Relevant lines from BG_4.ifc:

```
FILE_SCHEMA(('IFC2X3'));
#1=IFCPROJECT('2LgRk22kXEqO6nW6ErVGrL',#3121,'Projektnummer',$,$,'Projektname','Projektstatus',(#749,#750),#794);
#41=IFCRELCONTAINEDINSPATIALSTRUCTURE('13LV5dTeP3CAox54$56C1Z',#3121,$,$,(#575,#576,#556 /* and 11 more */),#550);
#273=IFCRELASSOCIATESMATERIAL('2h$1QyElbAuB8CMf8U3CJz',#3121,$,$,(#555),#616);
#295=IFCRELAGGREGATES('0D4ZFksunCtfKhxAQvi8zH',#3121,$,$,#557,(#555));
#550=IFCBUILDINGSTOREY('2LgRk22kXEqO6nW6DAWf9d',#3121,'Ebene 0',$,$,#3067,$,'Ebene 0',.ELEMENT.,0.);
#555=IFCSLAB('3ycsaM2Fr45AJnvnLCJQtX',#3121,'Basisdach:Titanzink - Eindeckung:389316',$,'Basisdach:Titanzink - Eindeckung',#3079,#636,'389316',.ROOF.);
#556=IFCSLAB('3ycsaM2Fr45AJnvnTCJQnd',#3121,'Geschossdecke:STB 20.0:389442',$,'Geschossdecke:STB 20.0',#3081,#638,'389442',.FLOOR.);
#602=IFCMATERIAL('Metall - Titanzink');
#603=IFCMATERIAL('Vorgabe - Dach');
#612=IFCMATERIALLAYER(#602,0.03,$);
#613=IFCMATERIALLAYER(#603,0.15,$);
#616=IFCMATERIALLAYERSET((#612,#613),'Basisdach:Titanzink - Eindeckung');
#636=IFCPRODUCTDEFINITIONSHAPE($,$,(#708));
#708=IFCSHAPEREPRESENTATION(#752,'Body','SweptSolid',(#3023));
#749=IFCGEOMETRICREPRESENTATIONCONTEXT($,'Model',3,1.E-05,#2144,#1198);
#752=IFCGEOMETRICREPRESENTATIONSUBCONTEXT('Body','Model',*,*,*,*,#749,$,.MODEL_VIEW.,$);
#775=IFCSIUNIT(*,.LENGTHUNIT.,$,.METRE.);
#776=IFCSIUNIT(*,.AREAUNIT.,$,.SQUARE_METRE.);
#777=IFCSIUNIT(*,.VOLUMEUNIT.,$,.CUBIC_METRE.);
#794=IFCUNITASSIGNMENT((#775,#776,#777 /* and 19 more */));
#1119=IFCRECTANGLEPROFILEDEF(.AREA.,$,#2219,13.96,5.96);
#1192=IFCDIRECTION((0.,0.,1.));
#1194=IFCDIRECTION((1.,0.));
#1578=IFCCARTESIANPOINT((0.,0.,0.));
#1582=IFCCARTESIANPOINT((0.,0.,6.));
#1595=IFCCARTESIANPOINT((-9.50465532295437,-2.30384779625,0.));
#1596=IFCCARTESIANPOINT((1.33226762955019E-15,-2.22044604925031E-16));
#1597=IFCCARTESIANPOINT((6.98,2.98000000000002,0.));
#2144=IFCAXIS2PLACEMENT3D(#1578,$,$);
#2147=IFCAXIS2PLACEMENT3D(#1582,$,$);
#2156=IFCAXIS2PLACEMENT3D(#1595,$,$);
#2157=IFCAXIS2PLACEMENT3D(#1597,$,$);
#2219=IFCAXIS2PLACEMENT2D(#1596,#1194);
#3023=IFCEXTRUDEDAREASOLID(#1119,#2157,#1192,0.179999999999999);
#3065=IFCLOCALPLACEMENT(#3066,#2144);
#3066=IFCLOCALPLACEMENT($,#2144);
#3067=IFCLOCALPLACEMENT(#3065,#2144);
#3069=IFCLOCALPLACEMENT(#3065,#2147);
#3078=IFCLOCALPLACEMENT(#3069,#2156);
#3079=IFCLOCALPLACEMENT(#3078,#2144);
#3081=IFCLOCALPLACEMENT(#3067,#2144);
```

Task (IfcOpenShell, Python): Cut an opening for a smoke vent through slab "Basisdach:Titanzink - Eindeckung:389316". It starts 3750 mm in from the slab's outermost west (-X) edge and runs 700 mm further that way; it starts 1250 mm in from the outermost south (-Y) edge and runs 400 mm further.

```python
import numpy as np
import ifcopenshell
import ifcopenshell.api.feature
import ifcopenshell.api.geometry
import ifcopenshell.api.root
import ifcopenshell.geom
import ifcopenshell.util.placement
import ifcopenshell.util.representation
import ifcopenshell.util.shape
import ifcopenshell.util.unit

model = ifcopenshell.open("BG_4.ifc")
unit_scale = ifcopenshell.util.unit.calculate_unit_scale(model)
settings = ifcopenshell.geom.settings()


def volume(element):
    """Net volume in cubic metres, openings subtracted."""
    shape = ifcopenshell.geom.create_shape(settings, element)
    return ifcopenshell.util.shape.get_volume(shape.geometry)


slab = model.by_guid("3ycsaM2Fr45AJnvnLCJQtX")
before = volume(slab)

# Extent in the slab's own axes, in metres. The edges named are its -X and -Y sides.
slab_shape = ifcopenshell.geom.create_shape(settings, slab)
vertices = ifcopenshell.util.shape.get_vertices(slab_shape.geometry)
x_min, y_min, bottom = vertices.min(axis=0)
top = vertices[:, 2].max()

opening = ifcopenshell.api.root.create_entity(model, ifc_class="IfcOpeningElement", name="Smoke vent opening")
context = ifcopenshell.util.representation.get_context(model, "Model", "Body", "MODEL_VIEW")
width, depth = 0.7, 0.4
outline = [(0.0, 0.0), (width, 0.0), (width, depth), (0.0, depth), (0.0, 0.0)]
# Overshoot both faces by 50 mm so the cut is clean.
shape = ifcopenshell.api.geometry.add_slab_representation(
    model, context=context, depth=top - bottom + 0.1, polyline=outline
)
ifcopenshell.api.geometry.assign_representation(model, product=opening, representation=shape)

matrix = ifcopenshell.util.placement.get_local_placement(slab.ObjectPlacement)
matrix[:, 3] = matrix @ np.append(np.array([x_min + 3.75, y_min + 1.25, bottom - 0.05]) / unit_scale, 1.0)
ifcopenshell.api.geometry.edit_object_placement(model, product=opening, matrix=matrix, is_si=False)
ifcopenshell.api.feature.add_feature(model, feature=opening, element=slab)

after = volume(slab)

print(f"slab volume {before:.3f} -> {after:.3f} m3")

model.write("BG_4_updated.ifc")
```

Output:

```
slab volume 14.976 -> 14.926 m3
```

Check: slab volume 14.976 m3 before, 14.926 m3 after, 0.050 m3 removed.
